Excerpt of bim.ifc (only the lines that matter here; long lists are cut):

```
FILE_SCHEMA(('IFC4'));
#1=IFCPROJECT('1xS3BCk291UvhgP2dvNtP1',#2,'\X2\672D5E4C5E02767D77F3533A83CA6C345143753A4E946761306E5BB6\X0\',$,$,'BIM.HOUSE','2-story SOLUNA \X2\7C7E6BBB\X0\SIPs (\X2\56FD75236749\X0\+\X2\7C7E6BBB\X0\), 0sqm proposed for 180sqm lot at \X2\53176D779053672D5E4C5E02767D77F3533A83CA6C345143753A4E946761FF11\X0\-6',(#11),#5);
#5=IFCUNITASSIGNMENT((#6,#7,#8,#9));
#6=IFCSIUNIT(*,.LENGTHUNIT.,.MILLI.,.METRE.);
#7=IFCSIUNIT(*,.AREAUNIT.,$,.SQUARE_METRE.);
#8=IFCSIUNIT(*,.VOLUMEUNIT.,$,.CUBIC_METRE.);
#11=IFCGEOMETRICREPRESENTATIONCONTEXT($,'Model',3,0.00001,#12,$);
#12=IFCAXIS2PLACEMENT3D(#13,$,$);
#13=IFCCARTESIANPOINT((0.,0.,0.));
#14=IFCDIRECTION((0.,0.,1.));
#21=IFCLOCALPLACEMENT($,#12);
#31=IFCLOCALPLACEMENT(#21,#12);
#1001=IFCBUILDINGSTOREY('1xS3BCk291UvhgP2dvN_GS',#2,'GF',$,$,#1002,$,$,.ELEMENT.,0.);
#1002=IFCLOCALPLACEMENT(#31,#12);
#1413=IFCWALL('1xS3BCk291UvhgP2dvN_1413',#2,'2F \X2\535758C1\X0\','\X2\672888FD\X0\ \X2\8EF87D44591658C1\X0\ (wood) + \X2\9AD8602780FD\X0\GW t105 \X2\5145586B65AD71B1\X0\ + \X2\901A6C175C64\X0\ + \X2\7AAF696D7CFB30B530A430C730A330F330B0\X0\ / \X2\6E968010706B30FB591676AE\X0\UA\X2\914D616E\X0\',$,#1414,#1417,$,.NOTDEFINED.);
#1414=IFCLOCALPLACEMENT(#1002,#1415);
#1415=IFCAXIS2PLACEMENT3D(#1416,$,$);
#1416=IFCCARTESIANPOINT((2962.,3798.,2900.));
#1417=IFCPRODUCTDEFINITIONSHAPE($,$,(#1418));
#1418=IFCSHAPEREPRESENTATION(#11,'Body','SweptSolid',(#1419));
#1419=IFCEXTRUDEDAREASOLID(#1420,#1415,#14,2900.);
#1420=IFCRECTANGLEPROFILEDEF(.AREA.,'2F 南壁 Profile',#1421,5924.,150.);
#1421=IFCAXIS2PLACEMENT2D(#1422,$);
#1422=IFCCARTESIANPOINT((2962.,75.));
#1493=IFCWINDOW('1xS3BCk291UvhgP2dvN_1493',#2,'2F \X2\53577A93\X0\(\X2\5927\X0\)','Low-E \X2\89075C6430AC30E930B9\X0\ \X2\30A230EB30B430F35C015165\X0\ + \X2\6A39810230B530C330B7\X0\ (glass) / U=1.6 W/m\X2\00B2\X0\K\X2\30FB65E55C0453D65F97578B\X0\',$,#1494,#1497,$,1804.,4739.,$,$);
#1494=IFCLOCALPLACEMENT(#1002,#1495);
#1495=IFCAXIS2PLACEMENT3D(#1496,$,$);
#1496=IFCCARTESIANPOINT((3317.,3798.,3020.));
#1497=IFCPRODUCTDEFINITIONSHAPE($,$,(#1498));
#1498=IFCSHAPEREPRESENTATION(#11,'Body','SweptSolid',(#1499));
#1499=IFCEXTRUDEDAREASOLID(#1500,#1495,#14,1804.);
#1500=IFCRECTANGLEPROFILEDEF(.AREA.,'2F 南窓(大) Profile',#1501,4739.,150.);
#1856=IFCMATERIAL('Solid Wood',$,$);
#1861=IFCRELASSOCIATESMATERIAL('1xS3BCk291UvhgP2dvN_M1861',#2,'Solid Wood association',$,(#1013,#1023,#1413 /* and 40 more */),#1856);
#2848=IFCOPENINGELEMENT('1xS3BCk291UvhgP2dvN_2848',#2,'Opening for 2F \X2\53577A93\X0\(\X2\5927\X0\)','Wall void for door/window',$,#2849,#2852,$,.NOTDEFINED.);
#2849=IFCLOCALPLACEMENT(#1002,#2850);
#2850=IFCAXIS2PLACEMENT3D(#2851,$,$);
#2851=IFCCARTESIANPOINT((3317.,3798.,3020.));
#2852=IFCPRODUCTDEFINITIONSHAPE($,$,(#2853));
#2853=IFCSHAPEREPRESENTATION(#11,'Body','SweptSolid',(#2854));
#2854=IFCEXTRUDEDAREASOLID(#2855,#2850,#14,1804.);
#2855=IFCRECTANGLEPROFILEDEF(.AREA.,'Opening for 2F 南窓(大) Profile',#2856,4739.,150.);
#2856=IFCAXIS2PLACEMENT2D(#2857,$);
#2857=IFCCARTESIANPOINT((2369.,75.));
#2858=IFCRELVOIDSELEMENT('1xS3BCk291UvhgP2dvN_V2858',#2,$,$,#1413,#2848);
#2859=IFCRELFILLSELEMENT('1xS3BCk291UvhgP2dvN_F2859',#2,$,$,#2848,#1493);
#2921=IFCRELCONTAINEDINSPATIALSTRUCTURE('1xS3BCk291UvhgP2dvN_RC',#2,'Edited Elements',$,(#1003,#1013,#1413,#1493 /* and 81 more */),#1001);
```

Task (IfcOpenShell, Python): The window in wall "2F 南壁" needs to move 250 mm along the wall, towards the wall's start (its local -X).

```python
import ifcopenshell
import ifcopenshell.api.geometry
import ifcopenshell.util.placement

model = ifcopenshell.open("bim.ifc")

window = model.by_guid("1xS3BCk291UvhgP2dvN_1493")
opening = window.FillsVoids[0].RelatingOpeningElement
wall = opening.VoidsElements[0].RelatingBuildingElement

wall_matrix = ifcopenshell.util.placement.get_local_placement(wall.ObjectPlacement)
shift = wall_matrix[:3, 0] * -250.0
before = ifcopenshell.util.placement.get_local_placement(window.ObjectPlacement)[:3, 3].copy()

# The window is not placed relative to its opening, so move both.
for product in (opening, window):
    matrix = ifcopenshell.util.placement.get_local_placement(product.ObjectPlacement)
    matrix[:3, 3] += shift
    ifcopenshell.api.geometry.edit_object_placement(model, product=product, matrix=matrix, is_si=False)

after = ifcopenshell.util.placement.get_local_placement(window.ObjectPlacement)[:3, 3]
print("window moved by", (after - before).round(3) + 0.0)

model.write("bim_edited.ifc")
```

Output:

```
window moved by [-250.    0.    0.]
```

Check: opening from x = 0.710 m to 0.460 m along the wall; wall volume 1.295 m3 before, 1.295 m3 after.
